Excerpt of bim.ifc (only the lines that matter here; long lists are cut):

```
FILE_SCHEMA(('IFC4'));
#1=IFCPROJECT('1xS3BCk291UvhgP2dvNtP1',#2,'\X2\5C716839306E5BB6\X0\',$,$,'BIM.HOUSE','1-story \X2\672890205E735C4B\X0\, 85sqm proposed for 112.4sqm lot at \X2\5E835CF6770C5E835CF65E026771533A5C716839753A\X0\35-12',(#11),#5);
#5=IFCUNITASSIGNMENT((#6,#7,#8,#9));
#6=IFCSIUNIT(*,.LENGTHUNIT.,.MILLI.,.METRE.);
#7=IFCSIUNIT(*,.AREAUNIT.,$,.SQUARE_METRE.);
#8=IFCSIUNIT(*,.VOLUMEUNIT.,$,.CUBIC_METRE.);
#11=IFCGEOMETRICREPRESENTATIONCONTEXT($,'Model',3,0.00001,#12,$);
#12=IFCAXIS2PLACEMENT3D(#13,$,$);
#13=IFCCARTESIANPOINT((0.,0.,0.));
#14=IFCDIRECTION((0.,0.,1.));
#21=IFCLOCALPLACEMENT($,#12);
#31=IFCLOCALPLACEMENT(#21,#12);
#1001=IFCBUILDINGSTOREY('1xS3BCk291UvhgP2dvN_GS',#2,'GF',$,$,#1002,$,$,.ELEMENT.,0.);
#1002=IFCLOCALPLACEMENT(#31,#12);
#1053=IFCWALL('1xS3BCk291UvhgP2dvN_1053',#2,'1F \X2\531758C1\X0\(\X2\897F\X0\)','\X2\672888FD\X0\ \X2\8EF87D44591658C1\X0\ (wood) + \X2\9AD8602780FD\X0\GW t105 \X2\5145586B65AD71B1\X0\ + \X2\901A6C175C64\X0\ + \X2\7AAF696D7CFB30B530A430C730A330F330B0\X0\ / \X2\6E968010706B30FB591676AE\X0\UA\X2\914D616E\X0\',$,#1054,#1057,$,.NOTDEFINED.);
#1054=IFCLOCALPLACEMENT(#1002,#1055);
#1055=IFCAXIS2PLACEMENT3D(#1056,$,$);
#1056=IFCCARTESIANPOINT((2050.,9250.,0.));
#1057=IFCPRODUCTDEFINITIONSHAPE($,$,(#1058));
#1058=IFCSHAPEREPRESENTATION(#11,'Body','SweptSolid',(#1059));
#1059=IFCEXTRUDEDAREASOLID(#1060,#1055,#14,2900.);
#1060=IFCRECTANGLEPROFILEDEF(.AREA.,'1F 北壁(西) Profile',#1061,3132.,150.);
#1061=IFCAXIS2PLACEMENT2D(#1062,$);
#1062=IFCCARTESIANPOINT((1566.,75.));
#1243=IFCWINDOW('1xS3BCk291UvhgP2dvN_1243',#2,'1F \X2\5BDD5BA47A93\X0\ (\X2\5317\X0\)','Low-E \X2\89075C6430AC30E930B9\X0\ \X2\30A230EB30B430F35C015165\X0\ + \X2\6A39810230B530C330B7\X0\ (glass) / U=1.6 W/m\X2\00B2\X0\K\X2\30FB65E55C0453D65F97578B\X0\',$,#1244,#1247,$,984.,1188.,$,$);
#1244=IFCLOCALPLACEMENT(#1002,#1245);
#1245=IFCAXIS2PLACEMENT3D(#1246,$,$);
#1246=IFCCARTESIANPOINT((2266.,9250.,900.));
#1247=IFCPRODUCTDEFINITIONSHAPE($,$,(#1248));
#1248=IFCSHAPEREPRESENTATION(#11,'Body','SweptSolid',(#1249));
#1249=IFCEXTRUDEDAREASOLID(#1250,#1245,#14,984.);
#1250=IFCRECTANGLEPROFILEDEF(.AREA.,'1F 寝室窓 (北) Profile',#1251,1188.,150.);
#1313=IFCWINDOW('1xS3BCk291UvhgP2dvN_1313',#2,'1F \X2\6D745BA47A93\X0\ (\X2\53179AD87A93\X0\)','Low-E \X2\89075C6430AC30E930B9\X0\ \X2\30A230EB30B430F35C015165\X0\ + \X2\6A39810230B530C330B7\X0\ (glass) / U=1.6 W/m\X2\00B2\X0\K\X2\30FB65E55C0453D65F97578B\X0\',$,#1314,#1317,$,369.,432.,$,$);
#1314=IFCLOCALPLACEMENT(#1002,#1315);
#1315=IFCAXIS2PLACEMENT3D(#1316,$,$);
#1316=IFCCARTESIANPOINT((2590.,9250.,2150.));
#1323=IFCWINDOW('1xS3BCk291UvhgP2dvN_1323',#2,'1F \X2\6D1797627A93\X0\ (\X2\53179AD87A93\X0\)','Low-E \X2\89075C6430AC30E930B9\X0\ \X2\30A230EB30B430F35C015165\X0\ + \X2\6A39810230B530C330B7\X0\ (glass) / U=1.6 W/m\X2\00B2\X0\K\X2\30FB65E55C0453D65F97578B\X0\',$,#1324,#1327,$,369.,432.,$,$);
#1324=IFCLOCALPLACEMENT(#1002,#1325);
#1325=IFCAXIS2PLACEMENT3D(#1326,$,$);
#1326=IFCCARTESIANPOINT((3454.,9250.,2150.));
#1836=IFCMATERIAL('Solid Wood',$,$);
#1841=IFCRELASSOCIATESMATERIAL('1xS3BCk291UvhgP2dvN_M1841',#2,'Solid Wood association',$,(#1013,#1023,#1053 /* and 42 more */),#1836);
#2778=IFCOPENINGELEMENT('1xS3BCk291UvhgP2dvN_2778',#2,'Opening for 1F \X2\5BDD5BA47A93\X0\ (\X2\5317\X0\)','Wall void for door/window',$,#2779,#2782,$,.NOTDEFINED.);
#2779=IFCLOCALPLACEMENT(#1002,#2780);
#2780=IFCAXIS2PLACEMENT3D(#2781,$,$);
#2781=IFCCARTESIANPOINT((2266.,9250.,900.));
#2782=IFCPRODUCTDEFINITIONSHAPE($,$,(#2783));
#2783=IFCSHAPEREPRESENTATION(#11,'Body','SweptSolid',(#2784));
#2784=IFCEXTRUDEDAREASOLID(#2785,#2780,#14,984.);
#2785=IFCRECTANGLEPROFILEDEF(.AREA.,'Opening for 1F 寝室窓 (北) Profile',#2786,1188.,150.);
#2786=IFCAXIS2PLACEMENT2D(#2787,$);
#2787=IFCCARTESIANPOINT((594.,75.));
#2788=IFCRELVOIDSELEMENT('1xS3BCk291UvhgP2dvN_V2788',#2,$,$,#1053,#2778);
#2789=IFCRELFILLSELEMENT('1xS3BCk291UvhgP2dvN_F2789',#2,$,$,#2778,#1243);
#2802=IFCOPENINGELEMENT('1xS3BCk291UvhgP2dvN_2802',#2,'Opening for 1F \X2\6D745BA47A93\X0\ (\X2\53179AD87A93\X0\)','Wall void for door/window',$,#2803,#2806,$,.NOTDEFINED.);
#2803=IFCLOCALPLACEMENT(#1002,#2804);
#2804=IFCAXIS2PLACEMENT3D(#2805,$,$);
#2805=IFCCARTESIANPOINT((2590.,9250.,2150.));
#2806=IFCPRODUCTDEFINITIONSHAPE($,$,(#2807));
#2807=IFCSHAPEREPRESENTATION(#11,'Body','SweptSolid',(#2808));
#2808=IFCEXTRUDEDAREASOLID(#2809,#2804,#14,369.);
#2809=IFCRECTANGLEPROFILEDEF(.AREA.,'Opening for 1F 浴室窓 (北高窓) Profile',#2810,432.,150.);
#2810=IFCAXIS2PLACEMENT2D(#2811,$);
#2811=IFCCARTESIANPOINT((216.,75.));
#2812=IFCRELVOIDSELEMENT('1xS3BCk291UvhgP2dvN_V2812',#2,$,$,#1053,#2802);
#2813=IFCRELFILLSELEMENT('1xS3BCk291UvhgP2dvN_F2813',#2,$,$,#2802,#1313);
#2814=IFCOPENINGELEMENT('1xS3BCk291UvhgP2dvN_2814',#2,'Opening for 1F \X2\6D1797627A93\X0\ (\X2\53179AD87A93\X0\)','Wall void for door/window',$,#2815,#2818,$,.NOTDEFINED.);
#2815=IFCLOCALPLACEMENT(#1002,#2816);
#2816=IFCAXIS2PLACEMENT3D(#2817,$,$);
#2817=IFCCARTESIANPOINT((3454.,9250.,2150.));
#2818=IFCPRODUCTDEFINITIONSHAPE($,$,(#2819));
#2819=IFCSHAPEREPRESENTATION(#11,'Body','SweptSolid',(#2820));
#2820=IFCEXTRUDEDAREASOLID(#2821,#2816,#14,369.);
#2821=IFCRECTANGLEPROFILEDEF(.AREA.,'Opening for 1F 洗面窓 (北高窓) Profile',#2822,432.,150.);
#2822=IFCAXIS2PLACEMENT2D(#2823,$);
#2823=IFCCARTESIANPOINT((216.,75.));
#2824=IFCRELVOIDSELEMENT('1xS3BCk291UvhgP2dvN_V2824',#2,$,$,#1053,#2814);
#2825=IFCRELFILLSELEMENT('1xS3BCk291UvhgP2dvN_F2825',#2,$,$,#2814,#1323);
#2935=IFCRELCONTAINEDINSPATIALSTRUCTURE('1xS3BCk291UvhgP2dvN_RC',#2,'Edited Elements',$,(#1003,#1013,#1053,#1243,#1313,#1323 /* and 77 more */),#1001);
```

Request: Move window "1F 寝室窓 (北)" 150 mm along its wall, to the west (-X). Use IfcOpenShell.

```python
import ifcopenshell
import ifcopenshell.api.geometry
import ifcopenshell.util.placement

model = ifcopenshell.open("bim.ifc")

window = model.by_guid("1xS3BCk291UvhgP2dvN_1243")
opening = window.FillsVoids[0].RelatingOpeningElement
wall = opening.VoidsElements[0].RelatingBuildingElement

wall_matrix = ifcopenshell.util.placement.get_local_placement(wall.ObjectPlacement)
shift = wall_matrix[:3, 0] * -150.0
before = ifcopenshell.util.placement.get_local_placement(window.ObjectPlacement)[:3, 3].copy()

# The window is not placed relative to its opening, so move both.
for product in (opening, window):
    matrix = ifcopenshell.util.placement.get_local_placement(product.ObjectPlacement)
    matrix[:3, 3] += shift
    ifcopenshell.api.geometry.edit_object_placement(model, product=product, matrix=matrix, is_si=False)

after = ifcopenshell.util.placement.get_local_placement(window.ObjectPlacement)[:3, 3]
print("window moved by", (after - before).round(3) + 0.0)

model.write("bim_v2.ifc")
```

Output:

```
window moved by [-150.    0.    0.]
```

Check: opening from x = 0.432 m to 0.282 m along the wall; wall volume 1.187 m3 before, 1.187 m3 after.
